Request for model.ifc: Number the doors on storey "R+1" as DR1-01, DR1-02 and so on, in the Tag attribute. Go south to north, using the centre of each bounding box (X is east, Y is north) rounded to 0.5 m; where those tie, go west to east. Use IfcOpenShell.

First a look at what the model holds.

```python
import ifcopenshell
import ifcopenshell.util.element
import ifcopenshell.util.placement

model = ifcopenshell.open("model.ifc")
print(model.schema)
storey = next(s for s in model.by_type("IfcBuildingStorey") if s.Name == "R+1")
doors = [e for e in ifcopenshell.util.element.get_decomposition(storey) if e.is_a("IfcDoor")]
for e in sorted(doors, key=lambda e: e.id()):
    origin = ifcopenshell.util.placement.get_local_placement(e.ObjectPlacement)[:3, 3]
    print(e.id(), e.Tag, e.Name, origin.round(2) + 0.0, sep=" | ")
```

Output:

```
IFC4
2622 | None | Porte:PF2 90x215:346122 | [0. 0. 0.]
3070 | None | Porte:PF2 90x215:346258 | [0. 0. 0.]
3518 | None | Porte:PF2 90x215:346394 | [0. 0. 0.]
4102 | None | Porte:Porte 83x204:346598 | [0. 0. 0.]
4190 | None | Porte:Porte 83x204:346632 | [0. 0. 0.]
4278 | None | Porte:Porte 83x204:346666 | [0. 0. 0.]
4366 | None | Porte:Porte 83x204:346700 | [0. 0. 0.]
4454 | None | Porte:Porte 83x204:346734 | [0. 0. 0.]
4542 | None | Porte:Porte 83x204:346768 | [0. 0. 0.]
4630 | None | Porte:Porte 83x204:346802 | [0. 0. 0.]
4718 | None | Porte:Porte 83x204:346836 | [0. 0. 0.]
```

```python
import ifcopenshell
import ifcopenshell.geom
import ifcopenshell.util.element
import ifcopenshell.util.shape

model = ifcopenshell.open("model.ifc")
settings = ifcopenshell.geom.settings()
settings.set("use-world-coords", True)


def centre(element):
    shape = ifcopenshell.geom.create_shape(settings, element)
    return ifcopenshell.util.shape.get_bbox_centroid(shape.geometry)


storey = next(s for s in model.by_type("IfcBuildingStorey") if s.Name == "R+1")
doors = [e for e in ifcopenshell.util.element.get_decomposition(storey) if e.is_a("IfcDoor")]

# Insertion points can sit at a corner or the storey origin, so sort by the geometry (in metres).
centres = {e: centre(e) for e in doors}
doors.sort(key=lambda e: (round(centres[e][1] / 0.5), centres[e][0]))

for i, e in enumerate(doors, start=1):
    number = f"DR1-{i:02d}"
    e.Tag = number
    print(e.id(), number)

model.write("model-out.ifc")
```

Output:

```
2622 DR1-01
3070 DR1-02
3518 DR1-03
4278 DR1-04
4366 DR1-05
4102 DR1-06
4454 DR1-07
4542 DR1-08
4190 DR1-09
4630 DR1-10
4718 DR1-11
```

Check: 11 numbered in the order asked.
